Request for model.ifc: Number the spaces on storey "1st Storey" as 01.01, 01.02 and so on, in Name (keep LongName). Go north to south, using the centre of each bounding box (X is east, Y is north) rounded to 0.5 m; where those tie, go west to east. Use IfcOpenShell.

First a look at what the model holds.

```python
import ifcopenshell
import ifcopenshell.util.element
import ifcopenshell.util.placement

model = ifcopenshell.open("model.ifc")
print(model.schema)
storey = next(s for s in model.by_type("IfcBuildingStorey") if s.Name == "1st Storey")
spaces = [e for e in ifcopenshell.util.element.get_decomposition(storey) if e.is_a("IfcSpace")]
for e in sorted(spaces, key=lambda e: e.id()):
    origin = ifcopenshell.util.placement.get_local_placement(e.ObjectPlacement)[:3, 3]
    print(e.id(), e.Name, e.LongName, origin.round(2) + 0.0, sep=" | ")
```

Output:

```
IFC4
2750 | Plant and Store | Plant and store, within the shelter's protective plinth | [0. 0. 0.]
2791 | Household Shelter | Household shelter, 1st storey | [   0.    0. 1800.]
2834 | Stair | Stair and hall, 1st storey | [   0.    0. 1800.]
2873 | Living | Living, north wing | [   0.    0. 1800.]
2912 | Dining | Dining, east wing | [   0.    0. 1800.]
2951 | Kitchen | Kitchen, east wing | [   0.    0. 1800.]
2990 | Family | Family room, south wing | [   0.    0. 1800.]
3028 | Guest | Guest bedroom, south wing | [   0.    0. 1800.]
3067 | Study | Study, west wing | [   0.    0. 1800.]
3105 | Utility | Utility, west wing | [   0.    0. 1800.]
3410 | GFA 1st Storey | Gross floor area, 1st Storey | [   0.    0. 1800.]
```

```python
import ifcopenshell
import ifcopenshell.geom
import ifcopenshell.util.element
import ifcopenshell.util.shape

model = ifcopenshell.open("model.ifc")
settings = ifcopenshell.geom.settings()
settings.set("use-world-coords", True)


def centre(element):
    shape = ifcopenshell.geom.create_shape(settings, element)
    return ifcopenshell.util.shape.get_bbox_centroid(shape.geometry)


storey = next(s for s in model.by_type("IfcBuildingStorey") if s.Name == "1st Storey")
spaces = [e for e in ifcopenshell.util.element.get_decomposition(storey) if e.is_a("IfcSpace")]

# Insertion points can sit at a corner or the storey origin, so sort by the geometry (in metres).
centres = {e: centre(e) for e in spaces}
spaces.sort(key=lambda e: (-round(centres[e][1] / 0.5), centres[e][0]))

for i, e in enumerate(spaces, start=1):
    number = f"01.{i:02d}"
    e.Name = number
    print(e.id(), number)

model.write("model_v2.ifc")
```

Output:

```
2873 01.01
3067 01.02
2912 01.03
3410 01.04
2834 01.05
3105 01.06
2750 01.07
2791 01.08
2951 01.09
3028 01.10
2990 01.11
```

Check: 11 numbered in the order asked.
